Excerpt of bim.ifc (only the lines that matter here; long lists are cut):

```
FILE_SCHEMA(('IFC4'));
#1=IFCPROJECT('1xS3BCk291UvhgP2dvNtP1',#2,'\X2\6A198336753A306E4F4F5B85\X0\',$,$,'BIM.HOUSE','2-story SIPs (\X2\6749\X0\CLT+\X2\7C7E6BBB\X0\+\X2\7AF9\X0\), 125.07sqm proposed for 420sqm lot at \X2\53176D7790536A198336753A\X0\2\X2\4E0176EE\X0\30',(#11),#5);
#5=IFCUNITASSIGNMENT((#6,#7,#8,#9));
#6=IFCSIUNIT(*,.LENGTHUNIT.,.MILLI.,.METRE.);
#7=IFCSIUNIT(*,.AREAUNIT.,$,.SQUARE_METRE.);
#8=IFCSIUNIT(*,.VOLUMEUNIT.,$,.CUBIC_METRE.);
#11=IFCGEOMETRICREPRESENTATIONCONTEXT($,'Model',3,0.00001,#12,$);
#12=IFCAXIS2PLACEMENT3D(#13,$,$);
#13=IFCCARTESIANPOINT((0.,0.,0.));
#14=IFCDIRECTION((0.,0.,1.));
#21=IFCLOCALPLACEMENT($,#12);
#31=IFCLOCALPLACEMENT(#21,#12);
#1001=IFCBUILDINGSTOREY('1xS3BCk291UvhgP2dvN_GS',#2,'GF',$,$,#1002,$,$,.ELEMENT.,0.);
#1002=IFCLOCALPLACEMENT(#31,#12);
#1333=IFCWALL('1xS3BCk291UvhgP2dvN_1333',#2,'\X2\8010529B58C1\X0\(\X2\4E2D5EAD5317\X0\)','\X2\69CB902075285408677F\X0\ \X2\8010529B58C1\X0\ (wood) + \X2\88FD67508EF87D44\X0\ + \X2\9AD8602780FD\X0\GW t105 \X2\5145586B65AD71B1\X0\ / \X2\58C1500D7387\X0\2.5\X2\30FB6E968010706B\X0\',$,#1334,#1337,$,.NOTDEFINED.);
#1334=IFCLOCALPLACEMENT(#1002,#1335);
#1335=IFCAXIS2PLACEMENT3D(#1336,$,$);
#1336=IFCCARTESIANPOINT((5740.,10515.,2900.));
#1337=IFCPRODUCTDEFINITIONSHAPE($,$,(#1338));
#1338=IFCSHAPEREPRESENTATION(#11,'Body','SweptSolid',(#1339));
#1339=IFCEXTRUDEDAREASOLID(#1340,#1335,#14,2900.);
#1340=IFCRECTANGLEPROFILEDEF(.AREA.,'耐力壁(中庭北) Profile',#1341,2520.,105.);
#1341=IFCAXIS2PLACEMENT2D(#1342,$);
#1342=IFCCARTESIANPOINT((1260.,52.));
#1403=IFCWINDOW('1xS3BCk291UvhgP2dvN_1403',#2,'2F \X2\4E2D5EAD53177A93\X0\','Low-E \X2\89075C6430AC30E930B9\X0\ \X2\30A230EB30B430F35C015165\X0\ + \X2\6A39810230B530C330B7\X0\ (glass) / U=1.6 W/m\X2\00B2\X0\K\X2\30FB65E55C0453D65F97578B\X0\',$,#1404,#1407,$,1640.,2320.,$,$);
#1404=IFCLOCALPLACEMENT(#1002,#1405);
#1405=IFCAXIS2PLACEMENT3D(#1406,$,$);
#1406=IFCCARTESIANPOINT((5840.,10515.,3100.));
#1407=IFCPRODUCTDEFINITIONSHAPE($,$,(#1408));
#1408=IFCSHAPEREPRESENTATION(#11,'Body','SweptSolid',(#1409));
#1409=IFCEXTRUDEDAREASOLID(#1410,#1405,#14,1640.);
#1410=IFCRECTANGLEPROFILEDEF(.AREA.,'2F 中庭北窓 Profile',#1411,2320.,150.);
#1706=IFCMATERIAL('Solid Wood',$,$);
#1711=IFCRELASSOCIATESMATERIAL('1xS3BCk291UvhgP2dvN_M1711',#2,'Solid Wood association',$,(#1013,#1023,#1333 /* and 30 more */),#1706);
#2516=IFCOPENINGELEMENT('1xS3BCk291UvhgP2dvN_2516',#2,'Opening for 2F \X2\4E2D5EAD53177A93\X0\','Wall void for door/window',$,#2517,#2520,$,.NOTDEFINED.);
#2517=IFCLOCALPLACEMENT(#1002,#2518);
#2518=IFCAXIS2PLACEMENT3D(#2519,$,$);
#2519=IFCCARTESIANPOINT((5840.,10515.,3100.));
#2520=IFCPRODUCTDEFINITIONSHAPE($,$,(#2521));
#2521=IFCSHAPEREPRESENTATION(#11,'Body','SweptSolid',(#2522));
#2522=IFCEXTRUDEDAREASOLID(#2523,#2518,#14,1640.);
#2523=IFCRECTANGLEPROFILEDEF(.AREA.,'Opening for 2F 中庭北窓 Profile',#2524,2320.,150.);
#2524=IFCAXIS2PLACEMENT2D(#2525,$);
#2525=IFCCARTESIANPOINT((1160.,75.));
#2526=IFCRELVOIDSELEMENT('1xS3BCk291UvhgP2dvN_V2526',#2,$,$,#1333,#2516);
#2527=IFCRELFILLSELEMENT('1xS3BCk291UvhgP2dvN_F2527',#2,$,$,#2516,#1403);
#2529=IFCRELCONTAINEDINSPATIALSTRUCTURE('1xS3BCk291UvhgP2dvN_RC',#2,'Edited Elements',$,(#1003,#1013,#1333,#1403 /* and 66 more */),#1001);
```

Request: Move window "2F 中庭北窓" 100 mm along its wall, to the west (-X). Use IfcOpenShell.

```python
import ifcopenshell
import ifcopenshell.api.geometry
import ifcopenshell.util.placement

model = ifcopenshell.open("bim.ifc")

window = model.by_guid("1xS3BCk291UvhgP2dvN_1403")
opening = window.FillsVoids[0].RelatingOpeningElement
wall = opening.VoidsElements[0].RelatingBuildingElement

wall_matrix = ifcopenshell.util.placement.get_local_placement(wall.ObjectPlacement)
shift = wall_matrix[:3, 0] * -100.0
before = ifcopenshell.util.placement.get_local_placement(window.ObjectPlacement)[:3, 3].copy()

# The window is not placed relative to its opening, so move both.
for product in (opening, window):
    matrix = ifcopenshell.util.placement.get_local_placement(product.ObjectPlacement)
    matrix[:3, 3] += shift
    ifcopenshell.api.geometry.edit_object_placement(model, product=product, matrix=matrix, is_si=False)

after = ifcopenshell.util.placement.get_local_placement(window.ObjectPlacement)[:3, 3]
print("window moved by", (after - before).round(3) + 0.0)

model.write("bim-out.ifc")
```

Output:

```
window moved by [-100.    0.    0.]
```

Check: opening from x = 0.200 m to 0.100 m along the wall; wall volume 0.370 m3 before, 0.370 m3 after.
